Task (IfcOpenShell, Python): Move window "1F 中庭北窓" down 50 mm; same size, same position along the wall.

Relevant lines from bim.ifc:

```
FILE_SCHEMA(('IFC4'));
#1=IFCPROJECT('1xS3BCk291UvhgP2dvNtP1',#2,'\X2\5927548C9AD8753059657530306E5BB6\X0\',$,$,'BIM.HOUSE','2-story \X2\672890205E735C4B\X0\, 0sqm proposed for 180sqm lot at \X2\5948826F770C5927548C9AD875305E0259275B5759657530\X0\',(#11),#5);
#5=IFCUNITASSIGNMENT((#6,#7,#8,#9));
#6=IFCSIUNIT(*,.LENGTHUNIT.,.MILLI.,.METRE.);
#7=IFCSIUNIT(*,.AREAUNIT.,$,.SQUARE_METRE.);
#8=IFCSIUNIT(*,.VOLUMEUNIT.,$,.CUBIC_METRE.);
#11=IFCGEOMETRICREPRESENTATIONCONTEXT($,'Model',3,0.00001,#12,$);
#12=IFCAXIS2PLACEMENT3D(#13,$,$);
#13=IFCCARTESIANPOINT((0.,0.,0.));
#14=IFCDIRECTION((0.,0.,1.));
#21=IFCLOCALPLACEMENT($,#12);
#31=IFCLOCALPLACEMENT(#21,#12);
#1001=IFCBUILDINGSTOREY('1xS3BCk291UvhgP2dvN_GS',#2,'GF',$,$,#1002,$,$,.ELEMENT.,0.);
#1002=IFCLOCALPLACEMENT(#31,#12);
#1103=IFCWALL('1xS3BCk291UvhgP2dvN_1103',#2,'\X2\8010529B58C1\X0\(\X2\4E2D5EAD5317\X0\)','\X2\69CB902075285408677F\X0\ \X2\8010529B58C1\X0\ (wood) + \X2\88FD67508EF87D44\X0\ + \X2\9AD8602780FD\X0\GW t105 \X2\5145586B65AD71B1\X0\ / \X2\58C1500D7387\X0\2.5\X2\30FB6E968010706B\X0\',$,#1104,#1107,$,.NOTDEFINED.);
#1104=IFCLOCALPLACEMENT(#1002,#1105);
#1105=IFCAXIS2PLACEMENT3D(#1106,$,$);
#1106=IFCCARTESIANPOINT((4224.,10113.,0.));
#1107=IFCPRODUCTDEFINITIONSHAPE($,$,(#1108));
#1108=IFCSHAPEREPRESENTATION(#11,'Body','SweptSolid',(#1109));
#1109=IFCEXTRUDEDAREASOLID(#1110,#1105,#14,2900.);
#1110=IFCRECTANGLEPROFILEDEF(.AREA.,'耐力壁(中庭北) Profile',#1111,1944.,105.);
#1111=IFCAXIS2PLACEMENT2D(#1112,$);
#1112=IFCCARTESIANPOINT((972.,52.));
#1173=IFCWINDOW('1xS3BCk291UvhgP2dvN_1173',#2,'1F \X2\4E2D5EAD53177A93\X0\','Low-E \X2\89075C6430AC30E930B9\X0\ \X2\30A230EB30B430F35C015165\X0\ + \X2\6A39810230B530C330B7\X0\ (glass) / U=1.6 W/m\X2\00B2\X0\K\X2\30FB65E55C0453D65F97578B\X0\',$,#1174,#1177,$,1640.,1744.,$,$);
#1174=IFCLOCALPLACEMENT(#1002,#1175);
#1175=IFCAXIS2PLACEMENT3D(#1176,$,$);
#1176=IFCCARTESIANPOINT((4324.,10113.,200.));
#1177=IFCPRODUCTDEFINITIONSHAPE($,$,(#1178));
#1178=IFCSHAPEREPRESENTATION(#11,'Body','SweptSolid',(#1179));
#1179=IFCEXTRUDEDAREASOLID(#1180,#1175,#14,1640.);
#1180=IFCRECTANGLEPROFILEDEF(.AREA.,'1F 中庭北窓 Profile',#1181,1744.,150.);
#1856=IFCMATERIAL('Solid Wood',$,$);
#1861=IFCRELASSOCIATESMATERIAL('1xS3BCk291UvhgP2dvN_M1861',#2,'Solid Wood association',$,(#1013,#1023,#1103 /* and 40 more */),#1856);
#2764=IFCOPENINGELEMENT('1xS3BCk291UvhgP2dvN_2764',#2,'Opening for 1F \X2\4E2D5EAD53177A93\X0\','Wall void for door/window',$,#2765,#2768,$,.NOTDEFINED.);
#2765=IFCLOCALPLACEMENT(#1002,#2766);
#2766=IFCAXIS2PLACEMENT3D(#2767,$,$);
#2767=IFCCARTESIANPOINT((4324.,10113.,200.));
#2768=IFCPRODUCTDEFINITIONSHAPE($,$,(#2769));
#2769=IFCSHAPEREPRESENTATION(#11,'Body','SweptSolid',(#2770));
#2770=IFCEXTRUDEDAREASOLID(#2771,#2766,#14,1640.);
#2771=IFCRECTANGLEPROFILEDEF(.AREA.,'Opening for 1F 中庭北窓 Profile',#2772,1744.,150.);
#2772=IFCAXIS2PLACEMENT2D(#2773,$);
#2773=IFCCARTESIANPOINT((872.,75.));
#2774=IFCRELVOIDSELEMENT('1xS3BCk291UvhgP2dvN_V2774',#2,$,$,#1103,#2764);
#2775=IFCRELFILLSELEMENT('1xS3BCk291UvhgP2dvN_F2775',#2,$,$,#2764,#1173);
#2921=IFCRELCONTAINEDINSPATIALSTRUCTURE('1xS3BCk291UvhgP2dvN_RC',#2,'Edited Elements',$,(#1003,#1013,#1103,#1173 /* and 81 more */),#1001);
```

```python
import numpy as np
import ifcopenshell
import ifcopenshell.api.geometry
import ifcopenshell.util.placement
import ifcopenshell.util.unit

model = ifcopenshell.open("bim.ifc")
unit_scale = ifcopenshell.util.unit.calculate_unit_scale(model)

window = model.by_guid("1xS3BCk291UvhgP2dvN_1173")
opening = window.FillsVoids[0].RelatingOpeningElement
dz = -0.05 / unit_scale

shift = np.array([0.0, 0.0, dz])
# The window is not placed relative to its opening, so move both.
for product in (opening, window):
    matrix = ifcopenshell.util.placement.get_local_placement(product.ObjectPlacement)
    matrix[:3, 3] += shift
    ifcopenshell.api.geometry.edit_object_placement(model, product=product, matrix=matrix, is_si=False)

print(f"moved by {dz * unit_scale:+.3f} m")

model.write("bim_updated.ifc")
```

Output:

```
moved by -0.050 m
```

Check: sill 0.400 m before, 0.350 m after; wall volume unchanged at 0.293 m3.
